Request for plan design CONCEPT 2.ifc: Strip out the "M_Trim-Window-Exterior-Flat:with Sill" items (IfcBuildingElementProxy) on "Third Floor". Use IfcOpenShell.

First a look at what the model holds.

```python
import ifcopenshell
import ifcopenshell.util.element

model = ifcopenshell.open("plan design CONCEPT 2.ifc")
print(model.schema)
storey = next(s for s in model.by_type("IfcBuildingStorey") if s.Name == "Third Floor")
proxies = [e for e in ifcopenshell.util.element.get_decomposition(storey) if e.is_a("IfcBuildingElementProxy")]
seen = {}
for e in proxies:
    element_type = ifcopenshell.util.element.get_type(e)
    name = element_type.Name if element_type not in (None, e) else None
    seen[name] = seen.get(name, 0) + 1
for name, count in sorted(seen.items(), key=str):
    print(count, "x", name)
```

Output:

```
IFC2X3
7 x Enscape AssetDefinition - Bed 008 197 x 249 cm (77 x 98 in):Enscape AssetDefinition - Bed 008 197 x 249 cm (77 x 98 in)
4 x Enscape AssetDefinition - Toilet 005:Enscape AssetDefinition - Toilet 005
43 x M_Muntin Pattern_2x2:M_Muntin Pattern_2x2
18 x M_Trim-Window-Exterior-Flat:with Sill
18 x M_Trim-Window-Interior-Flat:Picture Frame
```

```python
import ifcopenshell
import ifcopenshell.api.root
import ifcopenshell.util.element

model = ifcopenshell.open("plan design CONCEPT 2.ifc")

storey = next(s for s in model.by_type("IfcBuildingStorey") if s.Name == "Third Floor")
proxies = [e for e in ifcopenshell.util.element.get_decomposition(storey) if e.is_a("IfcBuildingElementProxy")]
targets = [e for e in proxies if (t := ifcopenshell.util.element.get_type(e)) not in (None, e) and t.Name == "M_Trim-Window-Exterior-Flat:with Sill"]

for e in targets:
    ifcopenshell.api.root.remove_product(model, product=e)
print(len(targets), "removed")

model.write("plan design CONCEPT 2_rev.ifc")
```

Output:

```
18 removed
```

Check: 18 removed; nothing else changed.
